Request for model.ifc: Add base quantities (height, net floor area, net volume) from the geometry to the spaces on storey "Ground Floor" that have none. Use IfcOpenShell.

First a look at what the model holds.

```python
import ifcopenshell
import ifcopenshell.util.element
import ifcopenshell.util.unit

model = ifcopenshell.open("model.ifc")
print(model.schema)
for unit_type in ("LENGTHUNIT", "AREAUNIT", "VOLUMEUNIT"):
    print(unit_type, ifcopenshell.util.unit.calculate_unit_scale(model, unit_type))
storey = next(s for s in model.by_type("IfcBuildingStorey") if s.Name == "Ground Floor")
spaces = [e for e in ifcopenshell.util.element.get_decomposition(storey) if e.is_a("IfcSpace")]
for e in sorted(spaces, key=lambda e: e.id()):
    print(e.id(), e.is_a(), e.Name, list(ifcopenshell.util.element.get_psets(e, qtos_only=True)), sep=" | ")
```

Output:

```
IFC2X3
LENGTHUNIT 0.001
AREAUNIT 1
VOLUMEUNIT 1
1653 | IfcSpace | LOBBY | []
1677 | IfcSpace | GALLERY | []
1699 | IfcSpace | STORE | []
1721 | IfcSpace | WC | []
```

```python
import ifcopenshell
import ifcopenshell.api.pset
import ifcopenshell.geom
import ifcopenshell.util.element
import ifcopenshell.util.shape
import ifcopenshell.util.unit

model = ifcopenshell.open("model.ifc")
unit_scale = ifcopenshell.util.unit.calculate_unit_scale(model)
area_scale = ifcopenshell.util.unit.calculate_unit_scale(model, "AREAUNIT")
volume_scale = ifcopenshell.util.unit.calculate_unit_scale(model, "VOLUMEUNIT")
settings = ifcopenshell.geom.settings()

storey = next(s for s in model.by_type("IfcBuildingStorey") if s.Name == "Ground Floor")
spaces = [e for e in ifcopenshell.util.element.get_decomposition(storey) if e.is_a("IfcSpace")]

for e in sorted(spaces, key=lambda e: e.id()):
    if ifcopenshell.util.element.get_psets(e, qtos_only=True, should_inherit=False):
        continue
    # Geometry comes back in metres, in the element's own axes.
    shape = ifcopenshell.geom.create_shape(settings, e)
    values = {
        "Height": ifcopenshell.util.shape.get_z(shape.geometry) / unit_scale,
        "NetFloorArea": ifcopenshell.util.shape.get_footprint_area(shape.geometry) / area_scale,
        "NetVolume": ifcopenshell.util.shape.get_volume(shape.geometry) / volume_scale,
    }
    qto = ifcopenshell.api.pset.add_qto(model, product=e, name="BaseQuantities")
    ifcopenshell.api.pset.edit_qto(model, qto=qto, properties=values)
    print(e.id(), {k: round(v, 3) for k, v in values.items()})

model.write("model-out.ifc")
```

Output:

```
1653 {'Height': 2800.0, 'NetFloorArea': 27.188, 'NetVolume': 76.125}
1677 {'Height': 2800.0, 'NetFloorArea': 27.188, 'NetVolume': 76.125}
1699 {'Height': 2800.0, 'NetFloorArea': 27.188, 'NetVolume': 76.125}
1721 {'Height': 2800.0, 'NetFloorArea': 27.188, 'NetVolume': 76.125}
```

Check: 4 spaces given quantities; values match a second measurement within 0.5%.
